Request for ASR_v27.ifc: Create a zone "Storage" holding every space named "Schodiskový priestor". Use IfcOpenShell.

First a look at what the model holds.

```python
import ifcopenshell

model = ifcopenshell.open("ASR_v27.ifc")
print(model.schema)
seen = {}
for space in model.by_type("IfcSpace"):
    seen[space.LongName] = seen.get(space.LongName, 0) + 1
for name, count in sorted(seen.items(), key=str):
    print(count, "x", name)
print("zones:", [z.Name for z in model.by_type("IfcZone")][:20])
```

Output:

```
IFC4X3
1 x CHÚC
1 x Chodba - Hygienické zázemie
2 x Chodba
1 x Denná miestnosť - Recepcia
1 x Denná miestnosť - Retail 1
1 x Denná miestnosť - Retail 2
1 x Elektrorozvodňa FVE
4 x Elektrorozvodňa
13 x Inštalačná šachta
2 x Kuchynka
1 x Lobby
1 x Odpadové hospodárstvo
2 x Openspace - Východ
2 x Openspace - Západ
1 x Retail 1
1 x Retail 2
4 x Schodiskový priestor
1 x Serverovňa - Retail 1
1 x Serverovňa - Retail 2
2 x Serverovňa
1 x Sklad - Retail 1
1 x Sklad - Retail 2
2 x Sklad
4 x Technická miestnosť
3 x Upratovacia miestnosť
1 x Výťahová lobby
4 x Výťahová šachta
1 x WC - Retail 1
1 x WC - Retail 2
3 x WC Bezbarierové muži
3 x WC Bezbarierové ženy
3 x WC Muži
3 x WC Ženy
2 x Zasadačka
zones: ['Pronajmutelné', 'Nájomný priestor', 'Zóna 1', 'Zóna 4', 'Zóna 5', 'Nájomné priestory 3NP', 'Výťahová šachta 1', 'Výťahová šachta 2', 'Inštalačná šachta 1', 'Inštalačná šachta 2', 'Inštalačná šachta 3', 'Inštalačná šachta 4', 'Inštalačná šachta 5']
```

```python
import ifcopenshell
import ifcopenshell.api.group
import ifcopenshell.api.root

model = ifcopenshell.open("ASR_v27.ifc")

names = {"Schodiskový priestor"}
spaces = [s for s in model.by_type("IfcSpace") if s.LongName in names]

zone = ifcopenshell.api.root.create_entity(model, ifc_class="IfcZone", name="Storage")
ifcopenshell.api.group.assign_group(model, products=spaces, group=zone)
print(len(spaces), "spaces in", zone.Name)

model.write("ASR_v27_updated.ifc")
```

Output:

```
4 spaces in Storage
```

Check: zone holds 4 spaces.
